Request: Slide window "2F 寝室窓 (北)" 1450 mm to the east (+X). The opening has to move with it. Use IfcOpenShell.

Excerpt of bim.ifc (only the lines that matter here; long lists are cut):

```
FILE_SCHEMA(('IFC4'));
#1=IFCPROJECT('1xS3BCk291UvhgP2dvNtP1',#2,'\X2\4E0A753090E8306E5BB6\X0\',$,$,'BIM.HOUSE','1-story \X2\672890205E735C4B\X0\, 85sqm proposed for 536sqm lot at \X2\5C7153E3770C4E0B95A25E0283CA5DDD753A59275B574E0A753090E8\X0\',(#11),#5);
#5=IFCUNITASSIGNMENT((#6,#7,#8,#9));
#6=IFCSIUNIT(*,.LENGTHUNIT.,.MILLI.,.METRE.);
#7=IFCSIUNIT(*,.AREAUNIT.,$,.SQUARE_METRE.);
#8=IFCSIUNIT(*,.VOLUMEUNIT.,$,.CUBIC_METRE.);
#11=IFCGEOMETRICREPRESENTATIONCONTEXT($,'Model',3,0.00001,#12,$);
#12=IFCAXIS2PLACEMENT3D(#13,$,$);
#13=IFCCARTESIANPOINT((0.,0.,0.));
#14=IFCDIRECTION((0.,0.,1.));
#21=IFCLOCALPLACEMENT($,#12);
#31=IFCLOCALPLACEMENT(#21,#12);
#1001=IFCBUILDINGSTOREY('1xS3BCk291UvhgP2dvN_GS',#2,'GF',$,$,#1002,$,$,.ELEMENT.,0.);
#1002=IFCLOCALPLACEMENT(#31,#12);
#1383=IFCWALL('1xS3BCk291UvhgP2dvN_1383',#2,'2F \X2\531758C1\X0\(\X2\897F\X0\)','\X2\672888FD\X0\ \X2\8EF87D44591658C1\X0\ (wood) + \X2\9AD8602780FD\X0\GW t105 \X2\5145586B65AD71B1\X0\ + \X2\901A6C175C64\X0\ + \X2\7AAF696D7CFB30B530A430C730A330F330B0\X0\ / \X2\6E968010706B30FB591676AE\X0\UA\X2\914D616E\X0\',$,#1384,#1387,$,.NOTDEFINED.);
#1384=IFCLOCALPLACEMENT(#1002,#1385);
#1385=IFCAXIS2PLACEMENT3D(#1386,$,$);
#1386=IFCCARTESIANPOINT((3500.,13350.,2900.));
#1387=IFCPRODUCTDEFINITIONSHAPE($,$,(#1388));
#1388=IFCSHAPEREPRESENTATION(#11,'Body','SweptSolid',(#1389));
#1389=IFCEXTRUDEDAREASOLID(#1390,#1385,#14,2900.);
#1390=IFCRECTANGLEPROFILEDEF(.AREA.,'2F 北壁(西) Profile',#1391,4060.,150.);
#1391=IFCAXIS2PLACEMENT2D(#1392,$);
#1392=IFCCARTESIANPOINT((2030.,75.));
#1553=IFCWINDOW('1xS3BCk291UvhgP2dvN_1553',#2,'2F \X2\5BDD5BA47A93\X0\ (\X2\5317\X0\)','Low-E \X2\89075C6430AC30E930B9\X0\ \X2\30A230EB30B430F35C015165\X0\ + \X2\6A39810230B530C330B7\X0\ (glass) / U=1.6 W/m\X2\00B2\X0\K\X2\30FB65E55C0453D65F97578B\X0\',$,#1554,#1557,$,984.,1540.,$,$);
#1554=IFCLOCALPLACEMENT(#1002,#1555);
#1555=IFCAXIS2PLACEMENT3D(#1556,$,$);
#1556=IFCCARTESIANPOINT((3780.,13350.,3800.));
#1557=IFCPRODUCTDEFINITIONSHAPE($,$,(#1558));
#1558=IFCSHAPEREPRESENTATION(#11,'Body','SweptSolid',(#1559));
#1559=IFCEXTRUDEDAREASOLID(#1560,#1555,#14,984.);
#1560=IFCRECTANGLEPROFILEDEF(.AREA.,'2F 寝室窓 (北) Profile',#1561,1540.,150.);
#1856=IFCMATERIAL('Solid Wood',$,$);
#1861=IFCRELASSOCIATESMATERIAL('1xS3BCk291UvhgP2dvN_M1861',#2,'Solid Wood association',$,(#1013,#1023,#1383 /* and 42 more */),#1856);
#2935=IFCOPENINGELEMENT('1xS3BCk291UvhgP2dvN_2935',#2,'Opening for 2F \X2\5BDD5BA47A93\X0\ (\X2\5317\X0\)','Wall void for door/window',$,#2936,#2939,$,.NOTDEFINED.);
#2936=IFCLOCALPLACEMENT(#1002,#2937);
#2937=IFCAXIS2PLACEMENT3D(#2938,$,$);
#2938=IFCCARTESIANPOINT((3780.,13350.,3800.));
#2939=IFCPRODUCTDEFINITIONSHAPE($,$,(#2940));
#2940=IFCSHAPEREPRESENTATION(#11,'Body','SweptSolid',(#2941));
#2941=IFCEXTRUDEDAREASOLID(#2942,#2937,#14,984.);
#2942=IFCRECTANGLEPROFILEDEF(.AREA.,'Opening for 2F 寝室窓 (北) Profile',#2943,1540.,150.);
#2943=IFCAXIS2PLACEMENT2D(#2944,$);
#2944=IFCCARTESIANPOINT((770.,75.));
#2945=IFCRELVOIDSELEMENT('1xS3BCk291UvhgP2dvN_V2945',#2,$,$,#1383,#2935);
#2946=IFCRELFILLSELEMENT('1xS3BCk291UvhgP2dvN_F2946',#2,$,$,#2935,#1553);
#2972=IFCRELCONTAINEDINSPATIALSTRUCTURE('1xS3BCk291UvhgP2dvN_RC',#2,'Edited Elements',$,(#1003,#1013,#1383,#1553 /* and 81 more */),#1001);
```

```python
import ifcopenshell
import ifcopenshell.api.geometry
import ifcopenshell.util.placement
import ifcopenshell.util.unit

model = ifcopenshell.open("bim.ifc")
unit_scale = ifcopenshell.util.unit.calculate_unit_scale(model)

window = model.by_id(1553)
opening = window.FillsVoids[0].RelatingOpeningElement
wall = opening.VoidsElements[0].RelatingBuildingElement

wall_matrix = ifcopenshell.util.placement.get_local_placement(wall.ObjectPlacement)
shift = wall_matrix[:3, 0] * 1.45 / unit_scale
before = ifcopenshell.util.placement.get_local_placement(window.ObjectPlacement)[:3, 3].copy()

# The window is not placed relative to its opening, so move both.
for product in (opening, window):
    matrix = ifcopenshell.util.placement.get_local_placement(product.ObjectPlacement)
    matrix[:3, 3] += shift
    ifcopenshell.api.geometry.edit_object_placement(model, product=product, matrix=matrix, is_si=False)

after = ifcopenshell.util.placement.get_local_placement(window.ObjectPlacement)[:3, 3]
print("window moved by", (after - before).round(3) + 0.0)

model.write("bim-out.ifc")
```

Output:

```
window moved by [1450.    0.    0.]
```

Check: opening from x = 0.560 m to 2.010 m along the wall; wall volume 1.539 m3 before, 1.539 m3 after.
